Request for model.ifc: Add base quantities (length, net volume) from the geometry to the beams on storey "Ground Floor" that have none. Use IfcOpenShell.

First a look at what the model holds.

```python
import ifcopenshell
import ifcopenshell.util.element
import ifcopenshell.util.unit

model = ifcopenshell.open("model.ifc")
print(model.schema)
for unit_type in ("LENGTHUNIT", "AREAUNIT", "VOLUMEUNIT"):
    print(unit_type, ifcopenshell.util.unit.calculate_unit_scale(model, unit_type))
storey = next(s for s in model.by_type("IfcBuildingStorey") if s.Name == "Ground Floor")
beams = [e for e in ifcopenshell.util.element.get_decomposition(storey) if e.is_a("IfcBeam")]
for e in sorted(beams, key=lambda e: e.id()):
    print(e.id(), e.is_a(), e.Name, list(ifcopenshell.util.element.get_psets(e, qtos_only=True)), sep=" | ")
```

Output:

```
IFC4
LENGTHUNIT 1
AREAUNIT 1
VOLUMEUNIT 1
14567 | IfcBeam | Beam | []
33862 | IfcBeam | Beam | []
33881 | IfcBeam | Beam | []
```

```python
import ifcopenshell
import ifcopenshell.api.pset
import ifcopenshell.geom
import ifcopenshell.util.element
import ifcopenshell.util.shape
import ifcopenshell.util.unit

model = ifcopenshell.open("model.ifc")
unit_scale = ifcopenshell.util.unit.calculate_unit_scale(model)
volume_scale = ifcopenshell.util.unit.calculate_unit_scale(model, "VOLUMEUNIT")
settings = ifcopenshell.geom.settings()

storey = next(s for s in model.by_type("IfcBuildingStorey") if s.Name == "Ground Floor")
beams = [e for e in ifcopenshell.util.element.get_decomposition(storey) if e.is_a("IfcBeam")]

for e in sorted(beams, key=lambda e: e.id()):
    if ifcopenshell.util.element.get_psets(e, qtos_only=True, should_inherit=False):
        continue
    # Geometry comes back in metres, in the element's own axes.
    shape = ifcopenshell.geom.create_shape(settings, e)
    values = {
        "Length": ifcopenshell.util.shape.get_max_xyz(shape.geometry) / unit_scale,
        "NetVolume": ifcopenshell.util.shape.get_volume(shape.geometry) / volume_scale,
    }
    qto = ifcopenshell.api.pset.add_qto(model, product=e, name="Qto_BeamBaseQuantities")
    ifcopenshell.api.pset.edit_qto(model, qto=qto, properties=values)
    print(e.id(), {k: round(v, 3) for k, v in values.items()})

model.write("model_edited.ifc")
```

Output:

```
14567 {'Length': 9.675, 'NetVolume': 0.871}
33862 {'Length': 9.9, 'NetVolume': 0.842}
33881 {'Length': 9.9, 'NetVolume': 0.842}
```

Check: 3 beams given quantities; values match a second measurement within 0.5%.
